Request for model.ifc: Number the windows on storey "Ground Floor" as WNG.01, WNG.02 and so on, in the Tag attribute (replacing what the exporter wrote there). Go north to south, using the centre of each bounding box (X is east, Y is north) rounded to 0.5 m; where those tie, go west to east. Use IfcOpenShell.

First a look at what the model holds.

```python
import ifcopenshell
import ifcopenshell.util.element
import ifcopenshell.util.placement

model = ifcopenshell.open("model.ifc")
print(model.schema)
storey = next(s for s in model.by_type("IfcBuildingStorey") if s.Name == "Ground Floor")
windows = [e for e in ifcopenshell.util.element.get_decomposition(storey) if e.is_a("IfcWindow")]
for e in sorted(windows, key=lambda e: e.id()):
    origin = ifcopenshell.util.placement.get_local_placement(e.ObjectPlacement)[:3, 3]
    print(e.id(), e.Tag, e.Name, origin.round(2) + 0.0, sep=" | ")
```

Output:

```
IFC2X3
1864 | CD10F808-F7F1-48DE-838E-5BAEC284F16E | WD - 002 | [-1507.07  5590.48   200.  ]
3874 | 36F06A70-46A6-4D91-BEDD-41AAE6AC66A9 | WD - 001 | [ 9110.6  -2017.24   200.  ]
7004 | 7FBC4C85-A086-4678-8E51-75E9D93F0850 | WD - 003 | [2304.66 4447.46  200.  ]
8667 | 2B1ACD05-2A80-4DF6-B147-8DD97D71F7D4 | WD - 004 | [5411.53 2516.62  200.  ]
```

```python
import ifcopenshell
import ifcopenshell.geom
import ifcopenshell.util.element
import ifcopenshell.util.shape

model = ifcopenshell.open("model.ifc")
settings = ifcopenshell.geom.settings()
settings.set("use-world-coords", True)


def centre(element):
    shape = ifcopenshell.geom.create_shape(settings, element)
    return ifcopenshell.util.shape.get_bbox_centroid(shape.geometry)


storey = next(s for s in model.by_type("IfcBuildingStorey") if s.Name == "Ground Floor")
windows = [e for e in ifcopenshell.util.element.get_decomposition(storey) if e.is_a("IfcWindow")]

# Insertion points can sit at a corner or the storey origin, so sort by the geometry (in metres).
centres = {e: centre(e) for e in windows}
windows.sort(key=lambda e: (-round(centres[e][1] / 0.5), centres[e][0]))

for i, e in enumerate(windows, start=1):
    number = f"WNG.{i:02d}"
    e.Tag = number
    print(e.id(), number)

model.write("model_rev.ifc")
```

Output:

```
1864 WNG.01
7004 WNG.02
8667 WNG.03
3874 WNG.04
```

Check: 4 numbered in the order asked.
